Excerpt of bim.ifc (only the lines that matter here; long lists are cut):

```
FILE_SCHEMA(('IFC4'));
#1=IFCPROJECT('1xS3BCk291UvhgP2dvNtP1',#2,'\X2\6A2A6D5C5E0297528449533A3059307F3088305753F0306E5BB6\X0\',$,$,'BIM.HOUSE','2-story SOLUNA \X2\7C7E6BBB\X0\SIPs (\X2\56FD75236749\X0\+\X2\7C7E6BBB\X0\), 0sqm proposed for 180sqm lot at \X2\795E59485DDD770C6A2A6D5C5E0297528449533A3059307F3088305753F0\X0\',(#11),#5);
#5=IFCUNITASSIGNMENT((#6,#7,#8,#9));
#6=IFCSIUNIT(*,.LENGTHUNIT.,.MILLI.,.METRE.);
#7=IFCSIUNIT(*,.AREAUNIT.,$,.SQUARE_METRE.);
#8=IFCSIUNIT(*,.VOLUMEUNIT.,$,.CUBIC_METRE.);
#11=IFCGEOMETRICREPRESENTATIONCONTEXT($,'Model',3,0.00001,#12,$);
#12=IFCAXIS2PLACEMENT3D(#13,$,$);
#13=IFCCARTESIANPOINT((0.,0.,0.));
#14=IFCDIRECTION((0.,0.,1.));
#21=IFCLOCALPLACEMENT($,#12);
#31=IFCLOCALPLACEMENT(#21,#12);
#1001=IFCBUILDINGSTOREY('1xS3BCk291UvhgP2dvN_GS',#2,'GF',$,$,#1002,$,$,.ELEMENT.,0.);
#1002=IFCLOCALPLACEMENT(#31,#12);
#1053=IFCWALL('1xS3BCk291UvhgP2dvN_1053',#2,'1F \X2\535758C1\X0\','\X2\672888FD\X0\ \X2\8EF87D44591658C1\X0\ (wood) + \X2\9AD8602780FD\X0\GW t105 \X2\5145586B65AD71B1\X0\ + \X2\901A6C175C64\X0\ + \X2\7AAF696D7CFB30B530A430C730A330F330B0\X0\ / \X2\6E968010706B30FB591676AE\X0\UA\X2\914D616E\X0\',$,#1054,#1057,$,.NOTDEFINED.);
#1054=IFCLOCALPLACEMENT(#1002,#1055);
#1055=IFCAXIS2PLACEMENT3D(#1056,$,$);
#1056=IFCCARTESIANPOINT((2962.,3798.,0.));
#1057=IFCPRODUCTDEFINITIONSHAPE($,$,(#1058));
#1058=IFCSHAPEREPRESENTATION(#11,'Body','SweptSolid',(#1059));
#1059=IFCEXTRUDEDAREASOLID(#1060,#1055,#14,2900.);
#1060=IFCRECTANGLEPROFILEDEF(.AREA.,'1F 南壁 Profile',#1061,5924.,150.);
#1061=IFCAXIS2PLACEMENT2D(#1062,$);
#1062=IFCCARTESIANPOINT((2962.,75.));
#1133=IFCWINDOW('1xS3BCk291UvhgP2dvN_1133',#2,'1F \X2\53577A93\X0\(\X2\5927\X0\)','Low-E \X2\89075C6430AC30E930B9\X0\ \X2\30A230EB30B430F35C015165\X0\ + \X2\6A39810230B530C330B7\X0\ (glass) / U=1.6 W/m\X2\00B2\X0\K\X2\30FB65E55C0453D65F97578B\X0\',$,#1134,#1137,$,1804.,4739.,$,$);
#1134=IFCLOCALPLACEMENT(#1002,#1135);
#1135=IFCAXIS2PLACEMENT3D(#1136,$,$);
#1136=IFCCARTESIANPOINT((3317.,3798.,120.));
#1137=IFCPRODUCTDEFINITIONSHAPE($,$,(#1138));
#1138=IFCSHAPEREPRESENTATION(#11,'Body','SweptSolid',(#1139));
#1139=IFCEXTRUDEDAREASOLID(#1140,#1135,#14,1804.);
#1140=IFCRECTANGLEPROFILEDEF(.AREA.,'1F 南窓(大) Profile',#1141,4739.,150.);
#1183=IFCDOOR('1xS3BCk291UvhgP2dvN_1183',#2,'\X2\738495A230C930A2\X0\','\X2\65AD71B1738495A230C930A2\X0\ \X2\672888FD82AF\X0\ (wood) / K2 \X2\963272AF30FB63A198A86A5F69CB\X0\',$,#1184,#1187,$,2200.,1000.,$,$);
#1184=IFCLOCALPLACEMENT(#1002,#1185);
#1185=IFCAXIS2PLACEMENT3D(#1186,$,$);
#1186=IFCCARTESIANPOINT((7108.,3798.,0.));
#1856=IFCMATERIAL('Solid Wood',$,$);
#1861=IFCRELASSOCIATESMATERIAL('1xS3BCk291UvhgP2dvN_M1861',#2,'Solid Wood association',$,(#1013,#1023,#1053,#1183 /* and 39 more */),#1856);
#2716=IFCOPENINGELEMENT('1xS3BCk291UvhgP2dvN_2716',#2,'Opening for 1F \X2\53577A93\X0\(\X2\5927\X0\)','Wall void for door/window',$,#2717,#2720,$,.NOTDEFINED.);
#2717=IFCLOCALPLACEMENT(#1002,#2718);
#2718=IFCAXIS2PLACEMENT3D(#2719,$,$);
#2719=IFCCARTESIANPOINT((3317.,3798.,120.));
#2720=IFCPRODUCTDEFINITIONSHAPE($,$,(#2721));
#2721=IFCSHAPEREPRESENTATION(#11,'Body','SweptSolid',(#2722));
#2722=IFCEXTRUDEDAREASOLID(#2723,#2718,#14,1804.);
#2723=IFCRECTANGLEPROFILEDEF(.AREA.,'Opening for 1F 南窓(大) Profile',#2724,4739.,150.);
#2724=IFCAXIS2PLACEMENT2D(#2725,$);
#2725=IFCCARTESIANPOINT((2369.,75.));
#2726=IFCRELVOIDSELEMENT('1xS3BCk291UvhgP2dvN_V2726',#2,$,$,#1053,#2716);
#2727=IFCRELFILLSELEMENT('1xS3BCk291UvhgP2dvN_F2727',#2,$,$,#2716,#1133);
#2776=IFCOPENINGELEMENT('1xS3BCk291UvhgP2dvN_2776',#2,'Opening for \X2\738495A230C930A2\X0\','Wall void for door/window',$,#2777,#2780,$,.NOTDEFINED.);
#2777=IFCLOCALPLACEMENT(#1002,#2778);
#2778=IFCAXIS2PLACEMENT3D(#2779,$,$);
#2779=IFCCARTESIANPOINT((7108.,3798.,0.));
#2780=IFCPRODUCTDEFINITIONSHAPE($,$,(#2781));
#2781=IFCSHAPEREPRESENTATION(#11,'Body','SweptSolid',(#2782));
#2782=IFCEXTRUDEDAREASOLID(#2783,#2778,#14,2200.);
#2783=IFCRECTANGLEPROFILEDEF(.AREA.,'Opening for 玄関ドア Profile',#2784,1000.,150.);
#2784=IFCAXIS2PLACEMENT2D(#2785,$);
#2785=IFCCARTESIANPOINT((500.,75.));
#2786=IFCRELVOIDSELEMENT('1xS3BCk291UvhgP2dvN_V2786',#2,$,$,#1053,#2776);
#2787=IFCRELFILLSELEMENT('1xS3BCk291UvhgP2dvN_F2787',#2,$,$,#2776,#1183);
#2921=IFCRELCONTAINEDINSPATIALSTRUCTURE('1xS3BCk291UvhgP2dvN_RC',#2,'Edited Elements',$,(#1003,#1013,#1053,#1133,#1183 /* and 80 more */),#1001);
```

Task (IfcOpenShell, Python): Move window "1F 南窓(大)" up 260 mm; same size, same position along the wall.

```python
import numpy as np
import ifcopenshell
import ifcopenshell.api.geometry
import ifcopenshell.util.placement
import ifcopenshell.util.unit

model = ifcopenshell.open("bim.ifc")
unit_scale = ifcopenshell.util.unit.calculate_unit_scale(model)

window = model.by_guid("1xS3BCk291UvhgP2dvN_1133")
opening = window.FillsVoids[0].RelatingOpeningElement
dz = 0.26 / unit_scale

shift = np.array([0.0, 0.0, dz])
# The window is not placed relative to its opening, so move both.
for product in (opening, window):
    matrix = ifcopenshell.util.placement.get_local_placement(product.ObjectPlacement)
    matrix[:3, 3] += shift
    ifcopenshell.api.geometry.edit_object_placement(model, product=product, matrix=matrix, is_si=False)

print(f"moved by {dz * unit_scale:+.3f} m")

model.write("bim-out.ifc")
```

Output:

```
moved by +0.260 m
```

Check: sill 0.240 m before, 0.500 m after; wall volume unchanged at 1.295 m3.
